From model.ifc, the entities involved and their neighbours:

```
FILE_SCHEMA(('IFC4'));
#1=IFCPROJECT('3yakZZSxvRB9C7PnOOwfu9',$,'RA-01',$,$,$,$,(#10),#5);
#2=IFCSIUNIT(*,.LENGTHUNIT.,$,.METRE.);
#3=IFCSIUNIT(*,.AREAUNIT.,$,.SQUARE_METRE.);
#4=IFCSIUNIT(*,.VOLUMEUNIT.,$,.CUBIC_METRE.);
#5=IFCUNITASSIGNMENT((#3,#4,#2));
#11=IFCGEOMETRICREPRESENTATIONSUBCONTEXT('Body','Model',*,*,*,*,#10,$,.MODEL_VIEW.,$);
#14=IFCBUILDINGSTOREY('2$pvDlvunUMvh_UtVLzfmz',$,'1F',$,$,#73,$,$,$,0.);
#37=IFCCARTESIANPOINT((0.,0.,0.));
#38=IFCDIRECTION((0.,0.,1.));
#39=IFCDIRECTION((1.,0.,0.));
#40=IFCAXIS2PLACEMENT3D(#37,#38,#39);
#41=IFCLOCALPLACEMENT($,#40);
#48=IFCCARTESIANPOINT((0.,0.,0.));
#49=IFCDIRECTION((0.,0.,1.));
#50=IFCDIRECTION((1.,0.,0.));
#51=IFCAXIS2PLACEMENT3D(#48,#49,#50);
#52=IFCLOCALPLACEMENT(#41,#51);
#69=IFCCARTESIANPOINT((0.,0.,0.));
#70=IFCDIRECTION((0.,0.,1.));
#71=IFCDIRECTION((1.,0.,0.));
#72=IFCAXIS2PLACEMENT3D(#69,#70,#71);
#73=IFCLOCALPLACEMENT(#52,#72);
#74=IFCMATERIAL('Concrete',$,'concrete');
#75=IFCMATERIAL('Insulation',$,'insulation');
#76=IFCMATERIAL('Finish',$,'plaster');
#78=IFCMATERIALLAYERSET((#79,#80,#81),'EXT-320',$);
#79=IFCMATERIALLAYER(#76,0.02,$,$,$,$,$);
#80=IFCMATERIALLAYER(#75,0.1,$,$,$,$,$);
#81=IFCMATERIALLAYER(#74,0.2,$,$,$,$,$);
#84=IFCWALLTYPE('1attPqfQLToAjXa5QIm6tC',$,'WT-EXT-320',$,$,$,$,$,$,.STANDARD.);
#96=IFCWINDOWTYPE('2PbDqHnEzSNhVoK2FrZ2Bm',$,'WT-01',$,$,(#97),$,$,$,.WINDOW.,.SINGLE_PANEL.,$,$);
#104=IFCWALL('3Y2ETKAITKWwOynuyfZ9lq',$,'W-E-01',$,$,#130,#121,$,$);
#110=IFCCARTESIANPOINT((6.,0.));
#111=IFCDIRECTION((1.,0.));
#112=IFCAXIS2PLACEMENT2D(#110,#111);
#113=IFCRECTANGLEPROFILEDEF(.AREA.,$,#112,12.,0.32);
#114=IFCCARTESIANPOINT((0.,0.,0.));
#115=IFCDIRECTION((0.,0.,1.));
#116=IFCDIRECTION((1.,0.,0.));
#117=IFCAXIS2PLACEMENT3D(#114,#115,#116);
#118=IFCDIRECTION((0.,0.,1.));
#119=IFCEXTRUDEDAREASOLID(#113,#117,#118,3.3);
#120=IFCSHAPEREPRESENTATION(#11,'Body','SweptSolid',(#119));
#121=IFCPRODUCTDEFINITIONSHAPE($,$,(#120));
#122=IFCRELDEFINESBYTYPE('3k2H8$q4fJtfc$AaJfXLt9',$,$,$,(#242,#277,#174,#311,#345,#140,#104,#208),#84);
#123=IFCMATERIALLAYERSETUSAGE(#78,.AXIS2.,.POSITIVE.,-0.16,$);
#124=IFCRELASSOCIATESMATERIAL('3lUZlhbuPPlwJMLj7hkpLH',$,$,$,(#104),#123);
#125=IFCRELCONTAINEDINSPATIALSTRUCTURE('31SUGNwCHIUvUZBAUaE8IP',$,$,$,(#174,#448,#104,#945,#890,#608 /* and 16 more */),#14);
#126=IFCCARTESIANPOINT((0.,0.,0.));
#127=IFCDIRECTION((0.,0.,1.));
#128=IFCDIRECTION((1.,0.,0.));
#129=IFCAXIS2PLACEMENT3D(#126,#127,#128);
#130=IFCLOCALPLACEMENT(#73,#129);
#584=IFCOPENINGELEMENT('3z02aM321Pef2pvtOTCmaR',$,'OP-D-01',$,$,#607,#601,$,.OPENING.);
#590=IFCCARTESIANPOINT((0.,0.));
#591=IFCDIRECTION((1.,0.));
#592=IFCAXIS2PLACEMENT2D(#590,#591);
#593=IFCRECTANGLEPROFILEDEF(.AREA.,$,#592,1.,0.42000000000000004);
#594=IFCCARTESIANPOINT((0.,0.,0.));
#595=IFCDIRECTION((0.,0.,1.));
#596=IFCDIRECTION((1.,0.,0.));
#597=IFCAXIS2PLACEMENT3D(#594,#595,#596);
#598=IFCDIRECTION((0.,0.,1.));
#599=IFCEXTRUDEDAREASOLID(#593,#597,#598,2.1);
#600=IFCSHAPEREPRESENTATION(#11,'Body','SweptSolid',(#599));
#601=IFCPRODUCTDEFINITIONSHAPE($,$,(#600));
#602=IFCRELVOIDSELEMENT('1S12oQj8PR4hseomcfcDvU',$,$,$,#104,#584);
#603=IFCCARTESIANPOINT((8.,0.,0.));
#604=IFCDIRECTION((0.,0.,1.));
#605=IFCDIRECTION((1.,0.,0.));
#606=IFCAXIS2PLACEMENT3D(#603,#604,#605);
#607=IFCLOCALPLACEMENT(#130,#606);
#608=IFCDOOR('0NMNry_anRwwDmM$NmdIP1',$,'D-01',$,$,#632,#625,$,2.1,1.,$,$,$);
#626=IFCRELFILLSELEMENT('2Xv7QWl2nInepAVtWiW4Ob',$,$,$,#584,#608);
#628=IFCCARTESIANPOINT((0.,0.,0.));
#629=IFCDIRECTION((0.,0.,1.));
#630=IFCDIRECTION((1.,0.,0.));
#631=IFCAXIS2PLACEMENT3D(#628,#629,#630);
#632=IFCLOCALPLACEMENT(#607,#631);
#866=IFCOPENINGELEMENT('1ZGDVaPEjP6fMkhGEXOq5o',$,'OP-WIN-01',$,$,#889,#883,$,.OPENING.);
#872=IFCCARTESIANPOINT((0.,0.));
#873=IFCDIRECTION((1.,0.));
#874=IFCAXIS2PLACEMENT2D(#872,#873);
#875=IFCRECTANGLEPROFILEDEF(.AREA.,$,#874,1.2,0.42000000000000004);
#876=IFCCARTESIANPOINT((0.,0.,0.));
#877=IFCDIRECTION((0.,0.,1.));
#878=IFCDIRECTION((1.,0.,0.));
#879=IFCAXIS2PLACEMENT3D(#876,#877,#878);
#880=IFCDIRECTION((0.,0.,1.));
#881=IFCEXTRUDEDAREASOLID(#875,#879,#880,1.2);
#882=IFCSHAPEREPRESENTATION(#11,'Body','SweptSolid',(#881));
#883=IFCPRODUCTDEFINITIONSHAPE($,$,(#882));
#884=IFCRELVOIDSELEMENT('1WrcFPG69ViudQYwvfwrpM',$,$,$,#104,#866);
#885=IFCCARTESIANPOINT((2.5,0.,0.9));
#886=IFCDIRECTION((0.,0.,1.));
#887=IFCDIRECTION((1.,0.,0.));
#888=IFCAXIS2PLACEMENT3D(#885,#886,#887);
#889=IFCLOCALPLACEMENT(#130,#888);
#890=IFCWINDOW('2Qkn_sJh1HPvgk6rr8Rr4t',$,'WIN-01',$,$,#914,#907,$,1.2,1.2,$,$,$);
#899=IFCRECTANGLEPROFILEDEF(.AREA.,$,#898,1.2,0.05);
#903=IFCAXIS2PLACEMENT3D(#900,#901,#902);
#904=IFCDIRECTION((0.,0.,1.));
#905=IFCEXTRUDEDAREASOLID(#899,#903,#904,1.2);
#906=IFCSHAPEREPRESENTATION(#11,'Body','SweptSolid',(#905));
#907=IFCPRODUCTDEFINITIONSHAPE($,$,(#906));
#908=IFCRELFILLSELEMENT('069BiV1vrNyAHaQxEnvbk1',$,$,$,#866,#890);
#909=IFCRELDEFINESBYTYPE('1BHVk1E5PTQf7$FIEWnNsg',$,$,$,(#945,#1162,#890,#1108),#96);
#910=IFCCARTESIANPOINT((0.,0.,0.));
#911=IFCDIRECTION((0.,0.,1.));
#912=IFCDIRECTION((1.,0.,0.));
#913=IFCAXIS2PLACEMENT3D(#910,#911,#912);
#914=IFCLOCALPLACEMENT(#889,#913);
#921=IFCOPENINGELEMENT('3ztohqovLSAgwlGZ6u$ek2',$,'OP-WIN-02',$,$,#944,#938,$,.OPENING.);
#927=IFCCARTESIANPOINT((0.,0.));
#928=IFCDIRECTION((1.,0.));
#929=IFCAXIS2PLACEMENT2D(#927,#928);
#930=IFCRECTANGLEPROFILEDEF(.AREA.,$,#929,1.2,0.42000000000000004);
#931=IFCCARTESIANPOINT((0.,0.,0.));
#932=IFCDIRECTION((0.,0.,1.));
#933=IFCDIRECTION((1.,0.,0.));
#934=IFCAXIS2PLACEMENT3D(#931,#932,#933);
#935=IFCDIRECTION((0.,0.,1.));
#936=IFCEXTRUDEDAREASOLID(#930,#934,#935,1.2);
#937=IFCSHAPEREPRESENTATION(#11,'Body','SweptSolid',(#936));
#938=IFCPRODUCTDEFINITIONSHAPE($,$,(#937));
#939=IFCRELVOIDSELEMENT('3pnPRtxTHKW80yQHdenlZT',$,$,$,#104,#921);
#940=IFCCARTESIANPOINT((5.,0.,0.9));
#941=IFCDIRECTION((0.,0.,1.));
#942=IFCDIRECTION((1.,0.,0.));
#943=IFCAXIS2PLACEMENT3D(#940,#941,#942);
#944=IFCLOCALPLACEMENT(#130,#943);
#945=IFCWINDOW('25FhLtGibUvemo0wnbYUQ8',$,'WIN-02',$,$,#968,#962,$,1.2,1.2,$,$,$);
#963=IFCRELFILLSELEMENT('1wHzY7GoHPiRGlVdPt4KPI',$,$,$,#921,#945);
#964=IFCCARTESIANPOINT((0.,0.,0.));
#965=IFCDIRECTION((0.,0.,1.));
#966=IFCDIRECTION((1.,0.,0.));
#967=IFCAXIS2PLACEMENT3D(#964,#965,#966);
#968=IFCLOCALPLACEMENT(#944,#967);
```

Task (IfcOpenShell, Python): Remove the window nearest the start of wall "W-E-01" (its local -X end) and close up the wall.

```python
import ifcopenshell
import ifcopenshell.api.feature
import ifcopenshell.api.root
import ifcopenshell.geom
import ifcopenshell.util.shape

model = ifcopenshell.open("model.ifc")
settings = ifcopenshell.geom.settings()


def volume(element):
    """Net volume in cubic metres, openings subtracted."""
    shape = ifcopenshell.geom.create_shape(settings, element)
    return ifcopenshell.util.shape.get_volume(shape.geometry)


window = model.by_guid("2Qkn_sJh1HPvgk6rr8Rr4t")
opening = window.FillsVoids[0].RelatingOpeningElement
wall = opening.VoidsElements[0].RelatingBuildingElement
before = volume(wall)

ifcopenshell.api.root.remove_product(model, product=window)
ifcopenshell.api.feature.remove_feature(model, feature=opening)

after = volume(wall)

print(f"wall volume {before:.3f} -> {after:.3f} m3")

model.write("model_rev.ifc")
```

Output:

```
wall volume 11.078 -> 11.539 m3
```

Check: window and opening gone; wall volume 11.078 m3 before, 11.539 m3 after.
